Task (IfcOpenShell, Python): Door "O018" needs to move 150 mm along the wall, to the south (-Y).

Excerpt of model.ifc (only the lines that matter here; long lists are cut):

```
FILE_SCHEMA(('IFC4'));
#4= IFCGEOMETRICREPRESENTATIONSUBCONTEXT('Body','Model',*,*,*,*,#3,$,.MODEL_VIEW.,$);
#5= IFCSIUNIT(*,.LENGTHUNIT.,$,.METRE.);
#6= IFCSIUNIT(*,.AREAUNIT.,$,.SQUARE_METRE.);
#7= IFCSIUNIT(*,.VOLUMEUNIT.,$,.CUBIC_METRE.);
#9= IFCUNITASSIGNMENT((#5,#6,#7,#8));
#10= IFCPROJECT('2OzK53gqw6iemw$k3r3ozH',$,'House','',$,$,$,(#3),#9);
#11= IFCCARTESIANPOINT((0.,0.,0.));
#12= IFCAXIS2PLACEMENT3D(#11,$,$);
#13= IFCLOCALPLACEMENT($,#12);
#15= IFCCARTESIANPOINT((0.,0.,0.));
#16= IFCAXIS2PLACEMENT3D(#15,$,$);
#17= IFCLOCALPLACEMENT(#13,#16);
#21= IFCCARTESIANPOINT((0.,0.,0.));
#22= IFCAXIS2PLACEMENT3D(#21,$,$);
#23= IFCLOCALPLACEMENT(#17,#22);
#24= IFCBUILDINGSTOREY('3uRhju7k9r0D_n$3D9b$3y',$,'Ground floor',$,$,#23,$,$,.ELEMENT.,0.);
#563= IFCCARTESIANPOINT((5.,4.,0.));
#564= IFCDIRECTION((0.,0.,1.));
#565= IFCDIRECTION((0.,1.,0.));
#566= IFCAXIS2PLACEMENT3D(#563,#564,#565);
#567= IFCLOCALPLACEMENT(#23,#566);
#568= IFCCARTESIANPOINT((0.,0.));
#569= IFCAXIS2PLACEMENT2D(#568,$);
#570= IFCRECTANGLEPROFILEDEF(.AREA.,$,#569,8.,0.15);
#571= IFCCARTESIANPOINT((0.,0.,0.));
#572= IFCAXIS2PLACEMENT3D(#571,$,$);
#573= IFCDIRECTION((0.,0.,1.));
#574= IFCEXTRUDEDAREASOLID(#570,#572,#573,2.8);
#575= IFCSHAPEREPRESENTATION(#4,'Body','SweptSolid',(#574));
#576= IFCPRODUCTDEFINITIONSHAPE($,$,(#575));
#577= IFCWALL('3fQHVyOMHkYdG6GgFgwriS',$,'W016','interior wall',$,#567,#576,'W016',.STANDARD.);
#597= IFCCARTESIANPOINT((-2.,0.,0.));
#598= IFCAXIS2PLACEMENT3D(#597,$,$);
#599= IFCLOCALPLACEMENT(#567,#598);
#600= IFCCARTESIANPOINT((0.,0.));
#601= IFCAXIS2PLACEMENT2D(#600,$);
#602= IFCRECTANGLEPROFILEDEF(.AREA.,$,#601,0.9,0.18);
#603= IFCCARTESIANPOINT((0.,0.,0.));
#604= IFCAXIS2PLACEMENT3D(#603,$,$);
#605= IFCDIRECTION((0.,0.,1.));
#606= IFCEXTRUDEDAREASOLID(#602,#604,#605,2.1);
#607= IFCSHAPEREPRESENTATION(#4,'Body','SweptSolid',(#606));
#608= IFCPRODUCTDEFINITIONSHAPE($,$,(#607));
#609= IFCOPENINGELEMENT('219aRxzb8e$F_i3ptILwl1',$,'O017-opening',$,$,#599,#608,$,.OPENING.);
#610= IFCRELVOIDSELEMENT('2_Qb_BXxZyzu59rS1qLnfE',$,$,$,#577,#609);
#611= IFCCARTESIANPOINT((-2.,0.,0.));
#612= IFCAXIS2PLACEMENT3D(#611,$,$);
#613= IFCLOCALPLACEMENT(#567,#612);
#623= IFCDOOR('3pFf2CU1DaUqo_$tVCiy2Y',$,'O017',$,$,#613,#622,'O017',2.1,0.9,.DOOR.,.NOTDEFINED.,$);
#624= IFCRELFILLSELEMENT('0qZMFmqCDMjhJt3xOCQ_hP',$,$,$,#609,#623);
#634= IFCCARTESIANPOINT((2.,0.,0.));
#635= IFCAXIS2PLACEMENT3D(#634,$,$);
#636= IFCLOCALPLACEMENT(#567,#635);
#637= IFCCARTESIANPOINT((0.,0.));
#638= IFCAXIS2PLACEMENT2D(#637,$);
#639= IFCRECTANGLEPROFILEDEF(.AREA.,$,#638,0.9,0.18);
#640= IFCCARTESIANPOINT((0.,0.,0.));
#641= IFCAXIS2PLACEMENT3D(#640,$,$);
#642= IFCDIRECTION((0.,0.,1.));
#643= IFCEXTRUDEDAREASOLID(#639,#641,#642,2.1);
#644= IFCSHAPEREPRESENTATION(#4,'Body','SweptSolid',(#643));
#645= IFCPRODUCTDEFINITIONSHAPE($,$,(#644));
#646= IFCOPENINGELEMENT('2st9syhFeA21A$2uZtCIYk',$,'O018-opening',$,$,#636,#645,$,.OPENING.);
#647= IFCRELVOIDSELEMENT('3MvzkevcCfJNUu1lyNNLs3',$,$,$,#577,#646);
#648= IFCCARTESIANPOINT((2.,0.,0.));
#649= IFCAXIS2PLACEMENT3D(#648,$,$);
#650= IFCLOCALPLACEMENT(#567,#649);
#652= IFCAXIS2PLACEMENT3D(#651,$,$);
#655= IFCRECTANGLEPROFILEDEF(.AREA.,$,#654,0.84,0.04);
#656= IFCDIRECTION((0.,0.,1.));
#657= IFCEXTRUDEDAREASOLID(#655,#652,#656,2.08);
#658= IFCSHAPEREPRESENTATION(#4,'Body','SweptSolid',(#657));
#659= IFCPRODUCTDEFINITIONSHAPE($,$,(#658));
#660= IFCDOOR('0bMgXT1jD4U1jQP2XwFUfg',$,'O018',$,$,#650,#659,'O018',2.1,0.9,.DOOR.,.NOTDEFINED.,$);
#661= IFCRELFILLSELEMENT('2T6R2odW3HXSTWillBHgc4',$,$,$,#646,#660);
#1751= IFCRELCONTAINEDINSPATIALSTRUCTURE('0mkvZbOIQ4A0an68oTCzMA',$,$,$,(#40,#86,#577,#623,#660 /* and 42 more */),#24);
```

```python
import ifcopenshell
import ifcopenshell.api.geometry
import ifcopenshell.util.placement

model = ifcopenshell.open("model.ifc")

door = model.by_id(660)
opening = door.FillsVoids[0].RelatingOpeningElement
wall = opening.VoidsElements[0].RelatingBuildingElement

wall_matrix = ifcopenshell.util.placement.get_local_placement(wall.ObjectPlacement)
shift = wall_matrix[:3, 0] * -0.15
before = ifcopenshell.util.placement.get_local_placement(door.ObjectPlacement)[:3, 3].copy()

# The door is not placed relative to its opening, so move both.
for product in (opening, door):
    matrix = ifcopenshell.util.placement.get_local_placement(product.ObjectPlacement)
    matrix[:3, 3] += shift
    ifcopenshell.api.geometry.edit_object_placement(model, product=product, matrix=matrix, is_si=False)

after = ifcopenshell.util.placement.get_local_placement(door.ObjectPlacement)[:3, 3]
print("door moved by", (after - before).round(3) + 0.0)

model.write("model_updated.ifc")
```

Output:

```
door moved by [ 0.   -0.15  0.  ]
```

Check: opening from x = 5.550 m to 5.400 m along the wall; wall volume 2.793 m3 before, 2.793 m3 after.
